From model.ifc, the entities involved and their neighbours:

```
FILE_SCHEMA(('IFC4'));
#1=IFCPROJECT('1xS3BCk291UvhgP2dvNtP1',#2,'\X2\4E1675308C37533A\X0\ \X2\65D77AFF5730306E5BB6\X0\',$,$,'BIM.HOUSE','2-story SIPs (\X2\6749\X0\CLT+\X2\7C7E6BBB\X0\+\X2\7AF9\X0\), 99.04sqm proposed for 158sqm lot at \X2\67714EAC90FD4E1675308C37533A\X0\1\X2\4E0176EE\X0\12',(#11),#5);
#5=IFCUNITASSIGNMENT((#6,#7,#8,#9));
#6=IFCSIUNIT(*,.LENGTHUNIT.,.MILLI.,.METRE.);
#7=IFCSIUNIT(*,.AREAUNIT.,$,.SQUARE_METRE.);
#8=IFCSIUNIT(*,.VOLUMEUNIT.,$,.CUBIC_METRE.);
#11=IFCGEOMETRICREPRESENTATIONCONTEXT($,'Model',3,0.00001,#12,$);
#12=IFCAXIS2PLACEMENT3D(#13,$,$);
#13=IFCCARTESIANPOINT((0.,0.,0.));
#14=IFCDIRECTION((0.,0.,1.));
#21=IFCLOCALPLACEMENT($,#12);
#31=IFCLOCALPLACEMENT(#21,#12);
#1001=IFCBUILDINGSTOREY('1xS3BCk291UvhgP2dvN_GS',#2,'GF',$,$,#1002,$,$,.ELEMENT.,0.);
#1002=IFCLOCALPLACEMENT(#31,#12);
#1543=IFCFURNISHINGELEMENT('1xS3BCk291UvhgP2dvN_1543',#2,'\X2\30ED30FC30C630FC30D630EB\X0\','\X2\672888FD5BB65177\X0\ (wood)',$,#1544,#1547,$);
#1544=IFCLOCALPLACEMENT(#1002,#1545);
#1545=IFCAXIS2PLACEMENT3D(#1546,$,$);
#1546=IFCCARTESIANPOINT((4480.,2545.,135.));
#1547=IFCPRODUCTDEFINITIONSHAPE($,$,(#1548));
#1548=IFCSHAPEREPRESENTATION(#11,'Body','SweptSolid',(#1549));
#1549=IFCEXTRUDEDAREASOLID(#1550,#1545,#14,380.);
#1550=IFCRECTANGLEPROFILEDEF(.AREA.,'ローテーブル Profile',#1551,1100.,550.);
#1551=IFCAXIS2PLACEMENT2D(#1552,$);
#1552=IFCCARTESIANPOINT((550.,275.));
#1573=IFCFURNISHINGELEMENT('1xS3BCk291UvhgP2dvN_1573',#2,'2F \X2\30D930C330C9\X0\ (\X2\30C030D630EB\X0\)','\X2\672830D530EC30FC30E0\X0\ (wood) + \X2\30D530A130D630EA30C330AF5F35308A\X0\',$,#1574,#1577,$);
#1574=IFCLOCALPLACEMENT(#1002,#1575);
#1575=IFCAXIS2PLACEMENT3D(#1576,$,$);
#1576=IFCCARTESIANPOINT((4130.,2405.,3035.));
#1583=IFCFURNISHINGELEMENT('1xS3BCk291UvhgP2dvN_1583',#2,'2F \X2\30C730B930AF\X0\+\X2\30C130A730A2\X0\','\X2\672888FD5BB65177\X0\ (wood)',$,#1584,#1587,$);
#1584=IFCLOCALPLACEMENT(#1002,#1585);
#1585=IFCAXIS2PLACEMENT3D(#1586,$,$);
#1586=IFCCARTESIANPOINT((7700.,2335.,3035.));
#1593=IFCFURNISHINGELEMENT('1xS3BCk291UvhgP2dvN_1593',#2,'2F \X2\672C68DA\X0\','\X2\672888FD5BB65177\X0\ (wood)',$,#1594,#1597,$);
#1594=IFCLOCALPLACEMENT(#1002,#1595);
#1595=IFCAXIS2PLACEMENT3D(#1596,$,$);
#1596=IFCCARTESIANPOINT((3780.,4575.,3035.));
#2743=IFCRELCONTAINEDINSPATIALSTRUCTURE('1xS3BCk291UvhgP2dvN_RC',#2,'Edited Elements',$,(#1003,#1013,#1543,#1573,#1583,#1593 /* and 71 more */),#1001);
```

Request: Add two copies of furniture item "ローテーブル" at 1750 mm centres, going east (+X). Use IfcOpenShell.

```python
import numpy as np
import ifcopenshell
import ifcopenshell.api.geometry
import ifcopenshell.api.root
import ifcopenshell.util.element
import ifcopenshell.util.placement
import ifcopenshell.util.unit

model = ifcopenshell.open("model.ifc")
unit_scale = ifcopenshell.util.unit.calculate_unit_scale(model)


def reuse_history(source, copy):
    """copy_class also copies each property set's owner history, people and application; keep the originals."""
    for rel in copy.IsDefinedBy:
        if rel.is_a("IfcRelDefinesByProperties") and (history := rel.RelatingPropertyDefinition.OwnerHistory):
            rel.RelatingPropertyDefinition.OwnerHistory = source.OwnerHistory
            ifcopenshell.util.element.remove_deep2(model, history)


source = model.by_guid("1xS3BCk291UvhgP2dvN_1543")
base = ifcopenshell.util.placement.get_local_placement(source.ObjectPlacement)
step = np.array([1.0, 0.0, 0.0]) * 1.75 / unit_scale

for i in range(1, 3):
    copy = ifcopenshell.api.root.copy_class(model, product=source)
    copy.Representation = ifcopenshell.util.element.copy_deep(
        model, source.Representation, exclude=["IfcGeometricRepresentationContext", "IfcRepresentationMap"]
    )
    reuse_history(source, copy)
    matrix = base.copy()
    matrix[:3, 3] += i * step
    print("added at", matrix[:3, 3].round(3) + 0.0)
    ifcopenshell.api.geometry.edit_object_placement(model, product=copy, matrix=matrix, is_si=False)

model.write("model-out.ifc")
```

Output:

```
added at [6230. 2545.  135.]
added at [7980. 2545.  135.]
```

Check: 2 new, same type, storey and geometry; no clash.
